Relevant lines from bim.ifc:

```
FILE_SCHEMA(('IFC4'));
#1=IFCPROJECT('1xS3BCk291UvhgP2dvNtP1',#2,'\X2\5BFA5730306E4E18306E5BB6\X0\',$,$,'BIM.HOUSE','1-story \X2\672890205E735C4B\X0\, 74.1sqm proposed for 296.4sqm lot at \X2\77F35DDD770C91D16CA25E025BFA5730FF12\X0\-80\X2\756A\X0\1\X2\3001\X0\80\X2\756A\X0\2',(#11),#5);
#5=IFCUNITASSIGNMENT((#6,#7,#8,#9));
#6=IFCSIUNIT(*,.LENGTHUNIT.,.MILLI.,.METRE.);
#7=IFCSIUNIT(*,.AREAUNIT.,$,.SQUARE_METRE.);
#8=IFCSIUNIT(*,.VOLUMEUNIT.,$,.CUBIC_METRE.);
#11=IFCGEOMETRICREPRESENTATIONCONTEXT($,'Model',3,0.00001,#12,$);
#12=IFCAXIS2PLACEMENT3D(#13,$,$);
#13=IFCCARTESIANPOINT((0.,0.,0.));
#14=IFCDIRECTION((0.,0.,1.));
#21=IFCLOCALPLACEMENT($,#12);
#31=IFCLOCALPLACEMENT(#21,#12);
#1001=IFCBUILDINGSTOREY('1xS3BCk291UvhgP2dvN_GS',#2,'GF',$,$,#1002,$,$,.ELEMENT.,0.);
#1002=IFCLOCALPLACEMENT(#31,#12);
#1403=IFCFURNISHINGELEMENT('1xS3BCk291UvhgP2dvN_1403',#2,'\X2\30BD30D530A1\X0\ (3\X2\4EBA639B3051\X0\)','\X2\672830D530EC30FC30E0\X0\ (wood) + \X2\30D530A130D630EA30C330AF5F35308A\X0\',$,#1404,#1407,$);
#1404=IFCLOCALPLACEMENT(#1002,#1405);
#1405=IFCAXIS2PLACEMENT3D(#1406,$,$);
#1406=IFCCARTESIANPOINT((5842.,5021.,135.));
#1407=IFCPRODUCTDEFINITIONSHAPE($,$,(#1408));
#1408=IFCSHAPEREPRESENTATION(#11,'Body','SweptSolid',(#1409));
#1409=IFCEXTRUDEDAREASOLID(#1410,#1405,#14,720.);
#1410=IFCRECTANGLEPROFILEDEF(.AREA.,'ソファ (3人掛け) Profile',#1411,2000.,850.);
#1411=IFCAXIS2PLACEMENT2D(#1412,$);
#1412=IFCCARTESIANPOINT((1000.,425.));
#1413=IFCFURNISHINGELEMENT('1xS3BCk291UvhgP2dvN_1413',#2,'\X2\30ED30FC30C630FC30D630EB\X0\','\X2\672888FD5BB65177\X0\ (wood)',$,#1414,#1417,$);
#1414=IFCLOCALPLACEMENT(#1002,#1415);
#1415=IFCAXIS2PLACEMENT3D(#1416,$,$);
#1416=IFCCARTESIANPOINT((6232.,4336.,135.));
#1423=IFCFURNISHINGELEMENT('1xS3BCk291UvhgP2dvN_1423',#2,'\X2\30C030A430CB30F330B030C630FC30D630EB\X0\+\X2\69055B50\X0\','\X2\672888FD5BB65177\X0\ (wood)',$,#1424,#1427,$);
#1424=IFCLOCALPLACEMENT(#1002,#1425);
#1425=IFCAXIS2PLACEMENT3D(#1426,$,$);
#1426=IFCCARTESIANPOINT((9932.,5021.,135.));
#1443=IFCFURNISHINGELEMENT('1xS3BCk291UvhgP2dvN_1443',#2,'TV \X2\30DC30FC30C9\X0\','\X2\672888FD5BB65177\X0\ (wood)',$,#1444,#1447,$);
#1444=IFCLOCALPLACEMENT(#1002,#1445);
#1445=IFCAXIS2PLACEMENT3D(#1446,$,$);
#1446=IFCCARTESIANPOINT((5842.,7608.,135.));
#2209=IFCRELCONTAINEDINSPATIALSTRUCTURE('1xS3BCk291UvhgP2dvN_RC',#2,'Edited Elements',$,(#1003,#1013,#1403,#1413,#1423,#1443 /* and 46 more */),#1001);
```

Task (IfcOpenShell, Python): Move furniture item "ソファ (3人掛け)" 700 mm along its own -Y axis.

```python
import ifcopenshell
import ifcopenshell.api.geometry
import ifcopenshell.util.placement

model = ifcopenshell.open("bim.ifc")

item = model.by_guid("1xS3BCk291UvhgP2dvN_1403")
matrix = ifcopenshell.util.placement.get_local_placement(item.ObjectPlacement)
matrix[:3, 3] -= matrix[:3, 1] * 700.0
ifcopenshell.api.geometry.edit_object_placement(model, product=item, matrix=matrix, is_si=False)

print(ifcopenshell.util.placement.get_local_placement(item.ObjectPlacement).round(3) + 0.0)

model.write("bim_v2.ifc")
```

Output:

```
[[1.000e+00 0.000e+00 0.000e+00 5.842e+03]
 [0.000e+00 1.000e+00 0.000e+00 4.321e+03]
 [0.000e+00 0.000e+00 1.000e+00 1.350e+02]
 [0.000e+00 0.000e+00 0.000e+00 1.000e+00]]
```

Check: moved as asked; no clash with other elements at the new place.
